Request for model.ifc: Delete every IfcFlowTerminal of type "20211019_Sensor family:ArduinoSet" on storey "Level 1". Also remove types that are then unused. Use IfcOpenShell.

First a look at what the model holds.

```python
import ifcopenshell
import ifcopenshell.util.element

model = ifcopenshell.open("model.ifc")
print(model.schema)
storey = next(s for s in model.by_type("IfcBuildingStorey") if s.Name == "Level 1")
terminals = [e for e in ifcopenshell.util.element.get_decomposition(storey) if e.is_a("IfcFlowTerminal")]
seen = {}
for e in terminals:
    element_type = ifcopenshell.util.element.get_type(e)
    name = element_type.Name if element_type not in (None, e) else None
    seen[name] = seen.get(name, 0) + 1
for name, count in sorted(seen.items(), key=str):
    print(count, "x", name)
```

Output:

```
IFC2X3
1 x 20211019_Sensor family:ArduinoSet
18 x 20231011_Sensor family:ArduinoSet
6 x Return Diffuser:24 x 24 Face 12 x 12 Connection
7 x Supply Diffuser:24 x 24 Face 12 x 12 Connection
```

```python
import ifcopenshell
import ifcopenshell.api.root
import ifcopenshell.util.element

model = ifcopenshell.open("model.ifc")

storey = next(s for s in model.by_type("IfcBuildingStorey") if s.Name == "Level 1")
terminals = [e for e in ifcopenshell.util.element.get_decomposition(storey) if e.is_a("IfcFlowTerminal")]
targets = [e for e in terminals if (t := ifcopenshell.util.element.get_type(e)) not in (None, e) and t.Name == "20211019_Sensor family:ArduinoSet"]
types = {ifcopenshell.util.element.get_type(e) for e in targets} - {None, *targets}

for e in targets:
    ifcopenshell.api.root.remove_product(model, product=e)
print(len(targets), "removed")

unused = [t for t in types if not ifcopenshell.util.element.get_types(t)]
for t in unused:
    ifcopenshell.api.root.remove_product(model, product=t)
print(len(unused), "unused types removed")

model.write("model_rev.ifc")
```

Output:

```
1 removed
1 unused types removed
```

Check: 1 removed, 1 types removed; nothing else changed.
